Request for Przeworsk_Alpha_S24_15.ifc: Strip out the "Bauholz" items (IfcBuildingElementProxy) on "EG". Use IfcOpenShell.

First a look at what the model holds.

```python
import ifcopenshell
import ifcopenshell.util.element

model = ifcopenshell.open("Przeworsk_Alpha_S24_15.ifc")
print(model.schema)
storey = next(s for s in model.by_type("IfcBuildingStorey") if s.Name == "EG")
proxies = [e for e in ifcopenshell.util.element.get_decomposition(storey) if e.is_a("IfcBuildingElementProxy")]
seen = {}
for e in proxies:
    element_type = ifcopenshell.util.element.get_type(e)
    name = element_type.Name if element_type not in (None, e) else None
    seen[name] = seen.get(name, 0) + 1
for name, count in sorted(seen.items(), key=str):
    print(count, "x", name)
```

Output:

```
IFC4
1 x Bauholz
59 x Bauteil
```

```python
import ifcopenshell
import ifcopenshell.api.root
import ifcopenshell.util.element

model = ifcopenshell.open("Przeworsk_Alpha_S24_15.ifc")

storey = next(s for s in model.by_type("IfcBuildingStorey") if s.Name == "EG")
proxies = [e for e in ifcopenshell.util.element.get_decomposition(storey) if e.is_a("IfcBuildingElementProxy")]
targets = [e for e in proxies if (t := ifcopenshell.util.element.get_type(e)) not in (None, e) and t.Name == "Bauholz"]

for e in targets:
    ifcopenshell.api.root.remove_product(model, product=e)
print(len(targets), "removed")

model.write("Przeworsk_Alpha_S24_15-out.ifc")
```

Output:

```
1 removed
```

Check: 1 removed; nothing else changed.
